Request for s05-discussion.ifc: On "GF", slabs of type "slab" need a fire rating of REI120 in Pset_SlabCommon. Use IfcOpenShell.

First a look at what the model holds.

```python
import ifcopenshell
import ifcopenshell.util.element

model = ifcopenshell.open("s05-discussion.ifc")
print(model.schema)
storey = next(s for s in model.by_type("IfcBuildingStorey") if s.Name == "GF")
slabs = [e for e in ifcopenshell.util.element.get_decomposition(storey) if e.is_a("IfcSlab")]
seen = {}
for e in slabs:
    element_type = ifcopenshell.util.element.get_type(e)
    key = (element_type.Name if element_type != e and element_type else None, ifcopenshell.util.element.get_pset(e, "Pset_SlabCommon", "FireRating"))
    seen[key] = seen.get(key, 0) + 1
for (name, value), count in sorted(seen.items(), key=str):
    print(count, "x", name, "|", value)
```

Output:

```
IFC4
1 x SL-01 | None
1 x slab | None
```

```python
import ifcopenshell
import ifcopenshell.api.pset
import ifcopenshell.util.element

model = ifcopenshell.open("s05-discussion.ifc")

storey = next(s for s in model.by_type("IfcBuildingStorey") if s.Name == "GF")
slabs = [e for e in ifcopenshell.util.element.get_decomposition(storey) if e.is_a("IfcSlab")]

count = 0
for e in slabs:
    element_type = ifcopenshell.util.element.get_type(e)
    if element_type in (None, e) or element_type.Name != "slab":
        continue
    # add_pset returns the element's existing set when there is one.
    pset = ifcopenshell.api.pset.add_pset(model, product=e, name="Pset_SlabCommon")
    ifcopenshell.api.pset.edit_pset(model, pset=pset, properties={"FireRating": "REI120"})
    count += 1

print(count, "slabs updated")

model.write("s05-discussion_rev.ifc")
```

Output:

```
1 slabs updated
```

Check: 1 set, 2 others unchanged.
